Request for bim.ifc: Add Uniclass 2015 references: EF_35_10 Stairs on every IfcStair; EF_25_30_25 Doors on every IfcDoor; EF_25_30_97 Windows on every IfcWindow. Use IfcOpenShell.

First a look at what the model holds.

```python
import ifcopenshell

model = ifcopenshell.open("bim.ifc")
print(model.schema)
print("classifications:", [c.Name for c in model.by_type("IfcClassification")])
for ifc_class in ("IfcDoor", "IfcRoof", "IfcStair", "IfcWall", "IfcWindow"):
    print(ifc_class, len(model.by_type(ifc_class)))
```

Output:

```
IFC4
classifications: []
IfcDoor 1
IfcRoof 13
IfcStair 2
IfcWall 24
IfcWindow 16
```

```python
import ifcopenshell
import ifcopenshell.api.classification

model = ifcopenshell.open("bim.ifc")

system = ifcopenshell.api.classification.add_classification(model, classification="Uniclass 2015")

codes = {
    "IfcStair": ("EF_35_10", "Stairs"),
    "IfcDoor": ("EF_25_30_25", "Doors"),
    "IfcWindow": ("EF_25_30_97", "Windows"),
}
for ifc_class, (code, name) in codes.items():
    products = model.by_type(ifc_class)
    ifcopenshell.api.classification.add_reference(
        model, products=products, classification=system, identification=code, name=name
    )
    print(code, len(products))

model.write("bim-out.ifc")
```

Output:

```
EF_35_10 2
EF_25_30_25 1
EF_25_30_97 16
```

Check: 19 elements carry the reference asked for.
